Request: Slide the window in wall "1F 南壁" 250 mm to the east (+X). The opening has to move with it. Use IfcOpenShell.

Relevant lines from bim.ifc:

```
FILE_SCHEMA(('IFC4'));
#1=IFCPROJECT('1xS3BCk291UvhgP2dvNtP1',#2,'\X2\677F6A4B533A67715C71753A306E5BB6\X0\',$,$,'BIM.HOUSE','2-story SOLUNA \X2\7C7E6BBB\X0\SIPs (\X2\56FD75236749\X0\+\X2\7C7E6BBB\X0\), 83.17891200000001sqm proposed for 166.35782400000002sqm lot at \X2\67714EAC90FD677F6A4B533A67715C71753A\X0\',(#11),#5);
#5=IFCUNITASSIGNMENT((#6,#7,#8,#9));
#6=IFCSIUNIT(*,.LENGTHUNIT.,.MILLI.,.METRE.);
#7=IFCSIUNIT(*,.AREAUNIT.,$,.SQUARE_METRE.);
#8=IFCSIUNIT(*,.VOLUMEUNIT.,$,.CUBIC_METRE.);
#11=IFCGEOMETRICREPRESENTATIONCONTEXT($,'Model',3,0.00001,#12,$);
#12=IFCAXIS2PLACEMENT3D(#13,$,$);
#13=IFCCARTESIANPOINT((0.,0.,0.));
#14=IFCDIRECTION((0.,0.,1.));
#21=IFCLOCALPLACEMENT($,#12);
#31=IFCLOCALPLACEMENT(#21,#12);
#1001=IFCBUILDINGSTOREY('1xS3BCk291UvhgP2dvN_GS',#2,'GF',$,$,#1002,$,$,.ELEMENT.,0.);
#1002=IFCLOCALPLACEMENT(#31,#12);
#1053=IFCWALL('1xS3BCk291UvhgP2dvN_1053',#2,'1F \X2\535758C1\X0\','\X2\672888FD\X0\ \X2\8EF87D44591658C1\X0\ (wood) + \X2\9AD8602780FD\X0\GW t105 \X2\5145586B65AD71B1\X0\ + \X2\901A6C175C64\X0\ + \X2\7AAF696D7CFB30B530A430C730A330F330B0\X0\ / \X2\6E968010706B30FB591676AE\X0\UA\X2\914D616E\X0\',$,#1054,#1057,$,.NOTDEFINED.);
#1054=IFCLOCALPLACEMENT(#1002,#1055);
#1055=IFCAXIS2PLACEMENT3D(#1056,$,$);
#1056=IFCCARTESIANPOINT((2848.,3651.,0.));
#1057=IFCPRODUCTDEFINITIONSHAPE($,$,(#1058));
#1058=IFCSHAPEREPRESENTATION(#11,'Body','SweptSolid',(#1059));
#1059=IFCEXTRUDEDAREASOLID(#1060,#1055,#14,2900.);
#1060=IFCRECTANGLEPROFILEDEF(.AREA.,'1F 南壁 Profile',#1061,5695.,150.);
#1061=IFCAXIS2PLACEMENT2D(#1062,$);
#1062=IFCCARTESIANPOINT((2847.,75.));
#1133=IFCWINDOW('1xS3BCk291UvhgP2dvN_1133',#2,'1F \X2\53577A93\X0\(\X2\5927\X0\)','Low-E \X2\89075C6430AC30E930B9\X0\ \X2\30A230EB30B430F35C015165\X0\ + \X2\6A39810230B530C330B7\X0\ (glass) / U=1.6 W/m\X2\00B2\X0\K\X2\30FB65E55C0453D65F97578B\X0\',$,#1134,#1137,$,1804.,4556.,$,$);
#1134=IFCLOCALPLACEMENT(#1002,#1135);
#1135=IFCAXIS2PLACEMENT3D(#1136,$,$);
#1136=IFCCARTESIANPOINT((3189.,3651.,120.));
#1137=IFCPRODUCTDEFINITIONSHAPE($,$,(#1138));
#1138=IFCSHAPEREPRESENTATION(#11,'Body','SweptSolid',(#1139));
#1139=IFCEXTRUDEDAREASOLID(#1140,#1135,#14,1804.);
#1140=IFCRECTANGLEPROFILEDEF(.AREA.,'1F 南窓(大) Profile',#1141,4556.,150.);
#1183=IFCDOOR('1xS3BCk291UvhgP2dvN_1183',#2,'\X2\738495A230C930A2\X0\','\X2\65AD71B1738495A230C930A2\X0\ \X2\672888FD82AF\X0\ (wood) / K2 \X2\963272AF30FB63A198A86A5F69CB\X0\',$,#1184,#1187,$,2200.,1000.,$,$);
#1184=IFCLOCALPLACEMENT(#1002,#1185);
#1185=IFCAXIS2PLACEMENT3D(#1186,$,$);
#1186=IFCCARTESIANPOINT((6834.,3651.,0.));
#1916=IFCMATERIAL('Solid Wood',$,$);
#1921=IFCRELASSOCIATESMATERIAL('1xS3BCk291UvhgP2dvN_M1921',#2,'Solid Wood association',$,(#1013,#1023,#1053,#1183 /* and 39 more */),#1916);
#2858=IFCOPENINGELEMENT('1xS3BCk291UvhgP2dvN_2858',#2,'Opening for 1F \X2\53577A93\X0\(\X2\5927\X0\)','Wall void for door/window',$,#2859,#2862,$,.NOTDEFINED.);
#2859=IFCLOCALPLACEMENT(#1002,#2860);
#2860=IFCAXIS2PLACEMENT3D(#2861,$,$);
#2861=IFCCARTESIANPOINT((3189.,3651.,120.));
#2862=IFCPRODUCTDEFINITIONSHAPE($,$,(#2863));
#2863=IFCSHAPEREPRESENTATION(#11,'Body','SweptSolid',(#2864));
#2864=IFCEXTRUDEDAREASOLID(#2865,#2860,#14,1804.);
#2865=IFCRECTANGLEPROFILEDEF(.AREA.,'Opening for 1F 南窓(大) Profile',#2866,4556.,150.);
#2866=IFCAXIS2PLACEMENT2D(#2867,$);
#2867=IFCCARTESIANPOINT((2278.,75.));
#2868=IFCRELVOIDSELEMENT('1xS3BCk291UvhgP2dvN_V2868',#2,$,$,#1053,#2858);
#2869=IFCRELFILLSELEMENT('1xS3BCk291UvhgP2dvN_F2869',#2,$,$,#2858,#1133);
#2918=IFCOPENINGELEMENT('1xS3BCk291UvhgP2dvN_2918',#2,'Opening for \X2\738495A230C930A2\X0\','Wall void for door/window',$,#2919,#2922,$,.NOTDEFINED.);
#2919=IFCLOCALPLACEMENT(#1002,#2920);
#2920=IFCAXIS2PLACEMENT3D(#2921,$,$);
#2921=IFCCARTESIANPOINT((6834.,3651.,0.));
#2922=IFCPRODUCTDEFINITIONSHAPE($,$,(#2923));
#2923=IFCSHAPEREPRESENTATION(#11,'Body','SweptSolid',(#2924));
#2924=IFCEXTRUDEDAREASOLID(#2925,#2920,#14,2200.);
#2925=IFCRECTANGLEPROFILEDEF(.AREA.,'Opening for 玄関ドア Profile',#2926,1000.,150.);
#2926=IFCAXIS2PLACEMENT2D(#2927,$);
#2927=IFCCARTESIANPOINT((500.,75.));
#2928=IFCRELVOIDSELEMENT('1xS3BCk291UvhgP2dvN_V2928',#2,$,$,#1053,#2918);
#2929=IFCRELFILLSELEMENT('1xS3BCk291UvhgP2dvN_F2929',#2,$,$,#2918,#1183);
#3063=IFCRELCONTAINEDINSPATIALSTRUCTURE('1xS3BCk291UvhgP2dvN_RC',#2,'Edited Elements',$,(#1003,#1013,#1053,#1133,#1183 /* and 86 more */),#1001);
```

```python
import ifcopenshell
import ifcopenshell.api.geometry
import ifcopenshell.util.placement
import ifcopenshell.util.unit

model = ifcopenshell.open("bim.ifc")
unit_scale = ifcopenshell.util.unit.calculate_unit_scale(model)

window = model.by_id(1133)
opening = window.FillsVoids[0].RelatingOpeningElement
wall = opening.VoidsElements[0].RelatingBuildingElement

wall_matrix = ifcopenshell.util.placement.get_local_placement(wall.ObjectPlacement)
shift = wall_matrix[:3, 0] * 0.25 / unit_scale
before = ifcopenshell.util.placement.get_local_placement(window.ObjectPlacement)[:3, 3].copy()

# The window is not placed relative to its opening, so move both.
for product in (opening, window):
    matrix = ifcopenshell.util.placement.get_local_placement(product.ObjectPlacement)
    matrix[:3, 3] += shift
    ifcopenshell.api.geometry.edit_object_placement(model, product=product, matrix=matrix, is_si=False)

after = ifcopenshell.util.placement.get_local_placement(window.ObjectPlacement)[:3, 3]
print("window moved by", (after - before).round(3) + 0.0)

model.write("bim_updated.ifc")
```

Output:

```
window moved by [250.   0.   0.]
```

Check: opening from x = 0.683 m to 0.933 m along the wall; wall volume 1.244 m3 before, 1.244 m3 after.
